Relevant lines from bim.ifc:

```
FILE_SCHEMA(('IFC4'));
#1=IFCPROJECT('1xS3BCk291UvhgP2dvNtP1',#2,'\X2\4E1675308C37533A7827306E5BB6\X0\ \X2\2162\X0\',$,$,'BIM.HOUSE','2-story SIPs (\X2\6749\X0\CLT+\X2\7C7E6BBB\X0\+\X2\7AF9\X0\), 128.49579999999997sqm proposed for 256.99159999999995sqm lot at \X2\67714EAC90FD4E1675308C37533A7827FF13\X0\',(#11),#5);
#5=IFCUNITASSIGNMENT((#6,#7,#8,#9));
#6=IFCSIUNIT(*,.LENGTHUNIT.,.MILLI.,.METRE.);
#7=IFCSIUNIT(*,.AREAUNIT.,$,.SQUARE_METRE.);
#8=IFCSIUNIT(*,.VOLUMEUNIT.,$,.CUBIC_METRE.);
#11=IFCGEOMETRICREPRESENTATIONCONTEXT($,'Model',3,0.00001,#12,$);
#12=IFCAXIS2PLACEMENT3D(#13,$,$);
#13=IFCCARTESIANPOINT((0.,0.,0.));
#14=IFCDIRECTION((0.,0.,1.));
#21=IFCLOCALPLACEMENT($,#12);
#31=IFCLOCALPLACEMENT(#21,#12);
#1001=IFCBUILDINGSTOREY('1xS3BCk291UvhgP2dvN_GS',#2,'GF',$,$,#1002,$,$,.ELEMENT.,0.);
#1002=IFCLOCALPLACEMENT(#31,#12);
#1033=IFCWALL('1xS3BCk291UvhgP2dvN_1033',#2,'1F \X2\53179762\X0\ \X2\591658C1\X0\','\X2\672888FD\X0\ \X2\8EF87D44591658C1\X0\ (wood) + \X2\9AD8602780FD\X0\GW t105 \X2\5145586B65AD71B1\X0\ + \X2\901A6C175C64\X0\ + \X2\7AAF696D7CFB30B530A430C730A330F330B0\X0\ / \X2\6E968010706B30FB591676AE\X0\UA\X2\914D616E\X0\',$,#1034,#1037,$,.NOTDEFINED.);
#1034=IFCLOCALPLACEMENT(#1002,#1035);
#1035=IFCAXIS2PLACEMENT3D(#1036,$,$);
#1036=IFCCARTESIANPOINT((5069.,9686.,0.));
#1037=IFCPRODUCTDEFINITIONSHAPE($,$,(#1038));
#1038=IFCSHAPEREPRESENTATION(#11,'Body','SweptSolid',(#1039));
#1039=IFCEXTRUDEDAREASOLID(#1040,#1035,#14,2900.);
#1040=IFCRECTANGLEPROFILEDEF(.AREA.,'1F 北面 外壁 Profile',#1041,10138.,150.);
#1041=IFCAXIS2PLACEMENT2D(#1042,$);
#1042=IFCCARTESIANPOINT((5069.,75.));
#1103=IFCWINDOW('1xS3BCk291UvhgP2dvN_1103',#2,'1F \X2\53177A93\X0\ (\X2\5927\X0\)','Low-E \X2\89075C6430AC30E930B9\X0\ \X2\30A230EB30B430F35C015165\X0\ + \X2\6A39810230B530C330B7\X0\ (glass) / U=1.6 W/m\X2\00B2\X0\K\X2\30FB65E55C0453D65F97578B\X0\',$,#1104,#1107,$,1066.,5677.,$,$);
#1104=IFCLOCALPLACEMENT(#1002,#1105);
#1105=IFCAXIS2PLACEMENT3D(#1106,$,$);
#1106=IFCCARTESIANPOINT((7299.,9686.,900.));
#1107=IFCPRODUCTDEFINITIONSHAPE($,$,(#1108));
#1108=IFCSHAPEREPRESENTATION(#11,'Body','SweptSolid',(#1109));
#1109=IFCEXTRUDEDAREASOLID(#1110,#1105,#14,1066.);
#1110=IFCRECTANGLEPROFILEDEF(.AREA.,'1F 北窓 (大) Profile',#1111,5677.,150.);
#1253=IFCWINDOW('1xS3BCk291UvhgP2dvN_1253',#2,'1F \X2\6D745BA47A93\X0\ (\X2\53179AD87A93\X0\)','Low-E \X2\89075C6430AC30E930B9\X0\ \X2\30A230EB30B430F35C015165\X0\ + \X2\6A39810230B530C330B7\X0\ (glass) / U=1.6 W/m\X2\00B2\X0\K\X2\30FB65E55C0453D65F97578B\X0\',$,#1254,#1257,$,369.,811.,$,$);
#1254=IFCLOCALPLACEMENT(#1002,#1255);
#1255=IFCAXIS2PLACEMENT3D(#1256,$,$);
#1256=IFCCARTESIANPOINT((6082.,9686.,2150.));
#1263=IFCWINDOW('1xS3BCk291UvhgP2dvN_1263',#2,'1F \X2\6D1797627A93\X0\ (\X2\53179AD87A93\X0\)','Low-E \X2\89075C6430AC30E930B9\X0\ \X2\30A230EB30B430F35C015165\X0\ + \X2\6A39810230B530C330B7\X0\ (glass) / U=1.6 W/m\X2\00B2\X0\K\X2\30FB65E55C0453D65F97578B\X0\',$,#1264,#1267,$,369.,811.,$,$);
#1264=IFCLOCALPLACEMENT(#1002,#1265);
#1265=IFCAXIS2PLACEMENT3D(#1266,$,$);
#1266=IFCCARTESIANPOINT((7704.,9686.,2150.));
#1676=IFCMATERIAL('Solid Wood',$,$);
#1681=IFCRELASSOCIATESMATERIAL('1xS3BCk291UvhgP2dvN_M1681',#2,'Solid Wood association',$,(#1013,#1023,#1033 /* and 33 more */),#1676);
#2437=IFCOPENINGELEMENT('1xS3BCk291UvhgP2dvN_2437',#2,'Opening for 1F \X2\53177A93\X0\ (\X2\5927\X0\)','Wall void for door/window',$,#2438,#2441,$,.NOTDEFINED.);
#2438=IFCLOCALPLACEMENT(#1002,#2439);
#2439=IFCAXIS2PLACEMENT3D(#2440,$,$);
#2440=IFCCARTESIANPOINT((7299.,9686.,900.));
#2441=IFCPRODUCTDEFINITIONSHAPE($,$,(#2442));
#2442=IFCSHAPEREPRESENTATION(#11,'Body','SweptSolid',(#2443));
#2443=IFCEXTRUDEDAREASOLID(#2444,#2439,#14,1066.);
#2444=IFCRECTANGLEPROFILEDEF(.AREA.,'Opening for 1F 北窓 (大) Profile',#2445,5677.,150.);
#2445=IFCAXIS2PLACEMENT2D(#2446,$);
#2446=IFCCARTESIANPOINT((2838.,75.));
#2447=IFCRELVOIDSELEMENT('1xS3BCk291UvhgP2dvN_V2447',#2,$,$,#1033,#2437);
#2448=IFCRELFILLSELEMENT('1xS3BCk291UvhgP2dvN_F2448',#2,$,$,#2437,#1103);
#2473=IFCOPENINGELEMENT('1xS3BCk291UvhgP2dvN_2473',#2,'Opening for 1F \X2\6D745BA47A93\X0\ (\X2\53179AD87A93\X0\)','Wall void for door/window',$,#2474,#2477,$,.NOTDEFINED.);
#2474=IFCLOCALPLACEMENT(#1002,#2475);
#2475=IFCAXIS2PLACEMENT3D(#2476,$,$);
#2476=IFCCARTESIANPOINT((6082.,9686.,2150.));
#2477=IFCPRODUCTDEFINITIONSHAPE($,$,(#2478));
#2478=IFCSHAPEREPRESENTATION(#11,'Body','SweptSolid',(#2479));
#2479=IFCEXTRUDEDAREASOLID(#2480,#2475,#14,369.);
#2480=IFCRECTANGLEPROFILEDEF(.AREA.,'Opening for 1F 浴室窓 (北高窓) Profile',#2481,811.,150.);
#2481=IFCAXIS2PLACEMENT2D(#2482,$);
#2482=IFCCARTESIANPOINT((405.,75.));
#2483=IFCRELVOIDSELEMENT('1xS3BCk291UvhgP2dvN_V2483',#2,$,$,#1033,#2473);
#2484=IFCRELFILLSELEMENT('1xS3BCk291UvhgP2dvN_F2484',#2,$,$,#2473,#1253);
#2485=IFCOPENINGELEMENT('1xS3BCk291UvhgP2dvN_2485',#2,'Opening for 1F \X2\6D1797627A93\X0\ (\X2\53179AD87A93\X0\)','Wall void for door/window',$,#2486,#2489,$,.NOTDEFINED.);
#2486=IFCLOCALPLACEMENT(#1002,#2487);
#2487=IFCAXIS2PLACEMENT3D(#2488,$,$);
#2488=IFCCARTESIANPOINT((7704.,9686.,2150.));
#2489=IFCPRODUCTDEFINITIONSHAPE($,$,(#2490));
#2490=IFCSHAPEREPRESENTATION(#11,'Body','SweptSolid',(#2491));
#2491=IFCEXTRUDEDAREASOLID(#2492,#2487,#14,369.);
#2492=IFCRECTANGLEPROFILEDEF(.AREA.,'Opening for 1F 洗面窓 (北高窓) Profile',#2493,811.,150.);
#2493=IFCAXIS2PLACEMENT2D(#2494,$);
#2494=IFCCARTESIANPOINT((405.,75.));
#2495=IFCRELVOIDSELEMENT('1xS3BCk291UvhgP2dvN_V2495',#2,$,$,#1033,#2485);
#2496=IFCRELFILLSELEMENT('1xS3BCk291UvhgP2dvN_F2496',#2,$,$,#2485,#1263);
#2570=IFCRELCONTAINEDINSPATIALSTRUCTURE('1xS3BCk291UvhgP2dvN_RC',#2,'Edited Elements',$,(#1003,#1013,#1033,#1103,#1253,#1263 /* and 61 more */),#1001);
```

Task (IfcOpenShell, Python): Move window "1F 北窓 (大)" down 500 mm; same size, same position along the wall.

```python
import numpy as np
import ifcopenshell
import ifcopenshell.api.geometry
import ifcopenshell.util.placement
import ifcopenshell.util.unit

model = ifcopenshell.open("bim.ifc")
unit_scale = ifcopenshell.util.unit.calculate_unit_scale(model)

window = model.by_guid("1xS3BCk291UvhgP2dvN_1103")
opening = window.FillsVoids[0].RelatingOpeningElement
dz = -500.0

shift = np.array([0.0, 0.0, dz])
# The window is not placed relative to its opening, so move both.
for product in (opening, window):
    matrix = ifcopenshell.util.placement.get_local_placement(product.ObjectPlacement)
    matrix[:3, 3] += shift
    ifcopenshell.api.geometry.edit_object_placement(model, product=product, matrix=matrix, is_si=False)

print(f"moved by {dz * unit_scale:+.3f} m")

model.write("bim_updated.ifc")
```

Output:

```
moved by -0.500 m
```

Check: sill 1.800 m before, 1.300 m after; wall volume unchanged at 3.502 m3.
